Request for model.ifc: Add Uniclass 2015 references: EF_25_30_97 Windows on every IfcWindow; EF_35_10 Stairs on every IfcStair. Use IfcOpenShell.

First a look at what the model holds.

```python
import ifcopenshell

model = ifcopenshell.open("model.ifc")
print(model.schema)
print("classifications:", [c.Name for c in model.by_type("IfcClassification")])
for ifc_class in ("IfcDoor", "IfcRoof", "IfcStair", "IfcWall", "IfcWindow"):
    print(ifc_class, len(model.by_type(ifc_class)))
```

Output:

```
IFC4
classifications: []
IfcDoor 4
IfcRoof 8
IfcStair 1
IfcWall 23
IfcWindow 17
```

```python
import ifcopenshell
import ifcopenshell.api.classification

model = ifcopenshell.open("model.ifc")

system = ifcopenshell.api.classification.add_classification(model, classification="Uniclass 2015")

codes = {
    "IfcWindow": ("EF_25_30_97", "Windows"),
    "IfcStair": ("EF_35_10", "Stairs"),
}
for ifc_class, (code, name) in codes.items():
    products = model.by_type(ifc_class)
    ifcopenshell.api.classification.add_reference(
        model, products=products, classification=system, identification=code, name=name
    )
    print(code, len(products))

model.write("model-out.ifc")
```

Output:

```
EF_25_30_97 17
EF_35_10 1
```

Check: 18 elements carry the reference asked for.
